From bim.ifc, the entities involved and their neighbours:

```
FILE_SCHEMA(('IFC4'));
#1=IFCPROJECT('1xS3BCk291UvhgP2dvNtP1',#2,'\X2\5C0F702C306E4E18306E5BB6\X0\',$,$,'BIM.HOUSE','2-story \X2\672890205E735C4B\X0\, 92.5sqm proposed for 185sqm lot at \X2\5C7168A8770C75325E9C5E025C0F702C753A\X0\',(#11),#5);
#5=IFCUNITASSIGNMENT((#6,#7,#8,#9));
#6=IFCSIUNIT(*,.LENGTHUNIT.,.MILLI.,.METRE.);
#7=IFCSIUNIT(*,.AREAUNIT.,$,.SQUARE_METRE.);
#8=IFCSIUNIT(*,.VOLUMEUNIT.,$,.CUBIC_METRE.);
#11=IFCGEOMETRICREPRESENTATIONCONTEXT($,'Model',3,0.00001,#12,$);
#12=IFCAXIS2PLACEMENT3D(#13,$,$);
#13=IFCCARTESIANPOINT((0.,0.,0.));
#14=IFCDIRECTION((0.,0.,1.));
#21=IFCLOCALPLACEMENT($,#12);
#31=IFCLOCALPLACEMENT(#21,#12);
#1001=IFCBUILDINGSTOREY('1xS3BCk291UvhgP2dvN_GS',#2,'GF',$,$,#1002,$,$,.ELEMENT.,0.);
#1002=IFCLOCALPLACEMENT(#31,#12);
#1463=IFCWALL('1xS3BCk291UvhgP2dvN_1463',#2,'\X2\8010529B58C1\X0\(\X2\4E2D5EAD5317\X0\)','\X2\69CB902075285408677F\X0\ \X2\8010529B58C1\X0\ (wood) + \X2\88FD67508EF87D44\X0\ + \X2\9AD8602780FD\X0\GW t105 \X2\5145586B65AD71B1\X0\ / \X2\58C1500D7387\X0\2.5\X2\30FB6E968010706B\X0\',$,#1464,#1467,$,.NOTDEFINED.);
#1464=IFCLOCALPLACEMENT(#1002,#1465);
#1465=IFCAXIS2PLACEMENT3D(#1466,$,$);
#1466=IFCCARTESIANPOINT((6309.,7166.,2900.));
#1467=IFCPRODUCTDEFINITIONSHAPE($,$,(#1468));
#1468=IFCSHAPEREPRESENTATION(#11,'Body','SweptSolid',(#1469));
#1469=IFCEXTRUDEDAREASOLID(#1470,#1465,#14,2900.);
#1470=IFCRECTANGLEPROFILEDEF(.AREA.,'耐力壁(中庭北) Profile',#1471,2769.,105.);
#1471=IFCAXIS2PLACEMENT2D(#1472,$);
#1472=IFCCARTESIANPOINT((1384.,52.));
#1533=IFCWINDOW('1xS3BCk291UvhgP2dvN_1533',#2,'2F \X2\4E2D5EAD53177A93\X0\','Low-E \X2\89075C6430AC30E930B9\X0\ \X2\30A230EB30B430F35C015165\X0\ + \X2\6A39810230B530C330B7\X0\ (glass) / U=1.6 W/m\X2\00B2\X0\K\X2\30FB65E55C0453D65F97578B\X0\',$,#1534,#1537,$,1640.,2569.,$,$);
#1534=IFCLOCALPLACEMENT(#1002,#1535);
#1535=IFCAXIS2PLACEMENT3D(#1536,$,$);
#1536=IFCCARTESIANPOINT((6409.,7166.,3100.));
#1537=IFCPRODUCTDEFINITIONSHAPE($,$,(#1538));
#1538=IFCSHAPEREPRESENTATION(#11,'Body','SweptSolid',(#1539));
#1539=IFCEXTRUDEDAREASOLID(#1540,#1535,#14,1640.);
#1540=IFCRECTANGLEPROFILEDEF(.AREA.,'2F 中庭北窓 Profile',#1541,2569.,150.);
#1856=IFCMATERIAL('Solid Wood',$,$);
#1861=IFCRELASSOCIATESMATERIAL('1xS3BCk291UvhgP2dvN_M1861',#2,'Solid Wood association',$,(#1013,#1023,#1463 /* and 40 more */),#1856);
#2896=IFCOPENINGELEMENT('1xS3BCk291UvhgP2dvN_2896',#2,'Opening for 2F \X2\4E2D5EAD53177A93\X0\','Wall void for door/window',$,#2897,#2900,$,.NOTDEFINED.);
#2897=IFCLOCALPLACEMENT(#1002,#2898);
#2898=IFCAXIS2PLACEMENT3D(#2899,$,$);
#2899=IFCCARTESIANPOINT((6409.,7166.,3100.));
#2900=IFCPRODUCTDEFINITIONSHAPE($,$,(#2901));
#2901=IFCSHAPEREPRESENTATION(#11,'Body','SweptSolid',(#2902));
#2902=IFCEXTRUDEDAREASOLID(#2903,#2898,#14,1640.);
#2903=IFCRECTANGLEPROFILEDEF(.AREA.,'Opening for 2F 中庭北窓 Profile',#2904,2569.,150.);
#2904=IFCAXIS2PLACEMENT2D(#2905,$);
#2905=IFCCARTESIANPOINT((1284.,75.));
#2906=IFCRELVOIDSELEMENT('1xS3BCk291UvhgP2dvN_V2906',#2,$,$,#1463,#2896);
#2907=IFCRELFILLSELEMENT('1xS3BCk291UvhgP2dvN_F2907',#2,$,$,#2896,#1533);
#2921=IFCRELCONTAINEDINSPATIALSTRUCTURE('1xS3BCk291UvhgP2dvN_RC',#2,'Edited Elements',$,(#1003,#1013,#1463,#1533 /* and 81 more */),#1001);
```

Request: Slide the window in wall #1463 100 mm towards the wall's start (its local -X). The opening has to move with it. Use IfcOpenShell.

```python
import ifcopenshell
import ifcopenshell.api.geometry
import ifcopenshell.util.placement
import ifcopenshell.util.unit

model = ifcopenshell.open("bim.ifc")
unit_scale = ifcopenshell.util.unit.calculate_unit_scale(model)

window = model.by_guid("1xS3BCk291UvhgP2dvN_1533")
opening = window.FillsVoids[0].RelatingOpeningElement
wall = opening.VoidsElements[0].RelatingBuildingElement

wall_matrix = ifcopenshell.util.placement.get_local_placement(wall.ObjectPlacement)
shift = wall_matrix[:3, 0] * -0.1 / unit_scale
before = ifcopenshell.util.placement.get_local_placement(window.ObjectPlacement)[:3, 3].copy()

# The window is not placed relative to its opening, so move both.
for product in (opening, window):
    matrix = ifcopenshell.util.placement.get_local_placement(product.ObjectPlacement)
    matrix[:3, 3] += shift
    ifcopenshell.api.geometry.edit_object_placement(model, product=product, matrix=matrix, is_si=False)

after = ifcopenshell.util.placement.get_local_placement(window.ObjectPlacement)[:3, 3]
print("window moved by", (after - before).round(3) + 0.0)

model.write("bim_v2.ifc")
```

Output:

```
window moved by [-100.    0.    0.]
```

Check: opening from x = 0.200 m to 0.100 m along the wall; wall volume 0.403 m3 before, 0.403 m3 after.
